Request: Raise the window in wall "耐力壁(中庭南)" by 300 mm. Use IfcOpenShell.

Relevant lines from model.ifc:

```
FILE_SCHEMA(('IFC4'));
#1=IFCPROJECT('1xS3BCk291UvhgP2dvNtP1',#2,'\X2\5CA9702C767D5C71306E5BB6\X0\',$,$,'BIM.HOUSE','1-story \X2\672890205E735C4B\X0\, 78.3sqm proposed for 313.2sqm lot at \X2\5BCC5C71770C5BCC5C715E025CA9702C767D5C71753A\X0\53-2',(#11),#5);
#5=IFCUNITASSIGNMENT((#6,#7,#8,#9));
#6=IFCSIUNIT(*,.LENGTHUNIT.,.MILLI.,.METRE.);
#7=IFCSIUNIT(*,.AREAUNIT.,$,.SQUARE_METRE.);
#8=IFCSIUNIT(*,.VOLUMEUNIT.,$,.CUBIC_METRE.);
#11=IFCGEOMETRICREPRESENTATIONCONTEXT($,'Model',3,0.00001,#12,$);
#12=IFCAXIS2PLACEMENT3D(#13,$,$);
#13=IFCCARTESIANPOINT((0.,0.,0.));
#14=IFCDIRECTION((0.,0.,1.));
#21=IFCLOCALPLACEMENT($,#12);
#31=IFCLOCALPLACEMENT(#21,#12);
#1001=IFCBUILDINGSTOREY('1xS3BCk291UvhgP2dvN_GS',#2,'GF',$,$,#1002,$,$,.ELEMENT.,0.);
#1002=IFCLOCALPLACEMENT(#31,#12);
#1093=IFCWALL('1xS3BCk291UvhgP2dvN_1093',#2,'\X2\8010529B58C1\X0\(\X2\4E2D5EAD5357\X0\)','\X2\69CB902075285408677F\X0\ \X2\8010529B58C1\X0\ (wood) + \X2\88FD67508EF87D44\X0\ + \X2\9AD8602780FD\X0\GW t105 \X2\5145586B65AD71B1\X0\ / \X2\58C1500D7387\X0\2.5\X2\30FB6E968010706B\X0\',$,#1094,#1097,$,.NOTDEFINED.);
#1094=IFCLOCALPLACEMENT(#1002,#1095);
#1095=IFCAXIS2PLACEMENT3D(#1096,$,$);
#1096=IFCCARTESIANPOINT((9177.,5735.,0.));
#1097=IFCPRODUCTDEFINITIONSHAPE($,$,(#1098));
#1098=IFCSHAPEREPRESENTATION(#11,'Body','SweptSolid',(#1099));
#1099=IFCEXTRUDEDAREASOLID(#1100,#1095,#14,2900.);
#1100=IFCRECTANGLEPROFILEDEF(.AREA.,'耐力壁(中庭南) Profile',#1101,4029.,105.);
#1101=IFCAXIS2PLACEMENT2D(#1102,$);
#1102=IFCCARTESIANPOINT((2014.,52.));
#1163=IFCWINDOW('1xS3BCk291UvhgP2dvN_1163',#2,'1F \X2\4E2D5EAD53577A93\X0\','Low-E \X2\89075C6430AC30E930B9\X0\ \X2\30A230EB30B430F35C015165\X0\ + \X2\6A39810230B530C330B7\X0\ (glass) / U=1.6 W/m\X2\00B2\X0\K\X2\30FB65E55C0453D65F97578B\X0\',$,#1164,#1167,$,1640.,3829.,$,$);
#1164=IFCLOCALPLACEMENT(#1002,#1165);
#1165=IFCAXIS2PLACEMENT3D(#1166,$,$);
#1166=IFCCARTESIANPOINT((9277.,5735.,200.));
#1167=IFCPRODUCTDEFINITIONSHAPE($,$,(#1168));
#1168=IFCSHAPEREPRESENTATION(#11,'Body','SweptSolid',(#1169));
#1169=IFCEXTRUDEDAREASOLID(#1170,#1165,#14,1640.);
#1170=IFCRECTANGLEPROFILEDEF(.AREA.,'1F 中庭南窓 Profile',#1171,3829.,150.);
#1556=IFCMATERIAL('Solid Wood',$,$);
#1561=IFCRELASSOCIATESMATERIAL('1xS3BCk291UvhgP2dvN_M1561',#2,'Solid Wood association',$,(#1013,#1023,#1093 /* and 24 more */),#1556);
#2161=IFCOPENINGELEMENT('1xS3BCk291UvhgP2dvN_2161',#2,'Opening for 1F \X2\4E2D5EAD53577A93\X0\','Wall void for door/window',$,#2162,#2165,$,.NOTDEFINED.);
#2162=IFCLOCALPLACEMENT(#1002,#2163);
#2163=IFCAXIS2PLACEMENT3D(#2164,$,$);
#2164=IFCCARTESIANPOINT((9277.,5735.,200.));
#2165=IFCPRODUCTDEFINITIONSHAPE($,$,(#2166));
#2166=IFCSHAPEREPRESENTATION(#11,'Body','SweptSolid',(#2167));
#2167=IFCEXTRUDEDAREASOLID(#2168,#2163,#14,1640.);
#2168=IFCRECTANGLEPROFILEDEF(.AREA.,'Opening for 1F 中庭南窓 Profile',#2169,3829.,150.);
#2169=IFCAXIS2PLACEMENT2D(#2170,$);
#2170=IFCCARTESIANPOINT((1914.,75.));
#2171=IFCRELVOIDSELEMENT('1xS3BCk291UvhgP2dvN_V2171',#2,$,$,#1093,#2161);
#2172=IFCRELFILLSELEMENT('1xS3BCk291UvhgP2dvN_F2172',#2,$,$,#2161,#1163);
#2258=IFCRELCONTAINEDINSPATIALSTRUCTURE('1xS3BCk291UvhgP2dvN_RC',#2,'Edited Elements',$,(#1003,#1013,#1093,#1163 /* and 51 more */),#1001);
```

```python
import numpy as np
import ifcopenshell
import ifcopenshell.api.geometry
import ifcopenshell.util.placement
import ifcopenshell.util.unit

model = ifcopenshell.open("model.ifc")
unit_scale = ifcopenshell.util.unit.calculate_unit_scale(model)

window = model.by_id(1163)
opening = window.FillsVoids[0].RelatingOpeningElement
dz = 0.3 / unit_scale

shift = np.array([0.0, 0.0, dz])
# The window is not placed relative to its opening, so move both.
for product in (opening, window):
    matrix = ifcopenshell.util.placement.get_local_placement(product.ObjectPlacement)
    matrix[:3, 3] += shift
    ifcopenshell.api.geometry.edit_object_placement(model, product=product, matrix=matrix, is_si=False)

print(f"moved by {dz * unit_scale:+.3f} m")

model.write("model-out.ifc")
```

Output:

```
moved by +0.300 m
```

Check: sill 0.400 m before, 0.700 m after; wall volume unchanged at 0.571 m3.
